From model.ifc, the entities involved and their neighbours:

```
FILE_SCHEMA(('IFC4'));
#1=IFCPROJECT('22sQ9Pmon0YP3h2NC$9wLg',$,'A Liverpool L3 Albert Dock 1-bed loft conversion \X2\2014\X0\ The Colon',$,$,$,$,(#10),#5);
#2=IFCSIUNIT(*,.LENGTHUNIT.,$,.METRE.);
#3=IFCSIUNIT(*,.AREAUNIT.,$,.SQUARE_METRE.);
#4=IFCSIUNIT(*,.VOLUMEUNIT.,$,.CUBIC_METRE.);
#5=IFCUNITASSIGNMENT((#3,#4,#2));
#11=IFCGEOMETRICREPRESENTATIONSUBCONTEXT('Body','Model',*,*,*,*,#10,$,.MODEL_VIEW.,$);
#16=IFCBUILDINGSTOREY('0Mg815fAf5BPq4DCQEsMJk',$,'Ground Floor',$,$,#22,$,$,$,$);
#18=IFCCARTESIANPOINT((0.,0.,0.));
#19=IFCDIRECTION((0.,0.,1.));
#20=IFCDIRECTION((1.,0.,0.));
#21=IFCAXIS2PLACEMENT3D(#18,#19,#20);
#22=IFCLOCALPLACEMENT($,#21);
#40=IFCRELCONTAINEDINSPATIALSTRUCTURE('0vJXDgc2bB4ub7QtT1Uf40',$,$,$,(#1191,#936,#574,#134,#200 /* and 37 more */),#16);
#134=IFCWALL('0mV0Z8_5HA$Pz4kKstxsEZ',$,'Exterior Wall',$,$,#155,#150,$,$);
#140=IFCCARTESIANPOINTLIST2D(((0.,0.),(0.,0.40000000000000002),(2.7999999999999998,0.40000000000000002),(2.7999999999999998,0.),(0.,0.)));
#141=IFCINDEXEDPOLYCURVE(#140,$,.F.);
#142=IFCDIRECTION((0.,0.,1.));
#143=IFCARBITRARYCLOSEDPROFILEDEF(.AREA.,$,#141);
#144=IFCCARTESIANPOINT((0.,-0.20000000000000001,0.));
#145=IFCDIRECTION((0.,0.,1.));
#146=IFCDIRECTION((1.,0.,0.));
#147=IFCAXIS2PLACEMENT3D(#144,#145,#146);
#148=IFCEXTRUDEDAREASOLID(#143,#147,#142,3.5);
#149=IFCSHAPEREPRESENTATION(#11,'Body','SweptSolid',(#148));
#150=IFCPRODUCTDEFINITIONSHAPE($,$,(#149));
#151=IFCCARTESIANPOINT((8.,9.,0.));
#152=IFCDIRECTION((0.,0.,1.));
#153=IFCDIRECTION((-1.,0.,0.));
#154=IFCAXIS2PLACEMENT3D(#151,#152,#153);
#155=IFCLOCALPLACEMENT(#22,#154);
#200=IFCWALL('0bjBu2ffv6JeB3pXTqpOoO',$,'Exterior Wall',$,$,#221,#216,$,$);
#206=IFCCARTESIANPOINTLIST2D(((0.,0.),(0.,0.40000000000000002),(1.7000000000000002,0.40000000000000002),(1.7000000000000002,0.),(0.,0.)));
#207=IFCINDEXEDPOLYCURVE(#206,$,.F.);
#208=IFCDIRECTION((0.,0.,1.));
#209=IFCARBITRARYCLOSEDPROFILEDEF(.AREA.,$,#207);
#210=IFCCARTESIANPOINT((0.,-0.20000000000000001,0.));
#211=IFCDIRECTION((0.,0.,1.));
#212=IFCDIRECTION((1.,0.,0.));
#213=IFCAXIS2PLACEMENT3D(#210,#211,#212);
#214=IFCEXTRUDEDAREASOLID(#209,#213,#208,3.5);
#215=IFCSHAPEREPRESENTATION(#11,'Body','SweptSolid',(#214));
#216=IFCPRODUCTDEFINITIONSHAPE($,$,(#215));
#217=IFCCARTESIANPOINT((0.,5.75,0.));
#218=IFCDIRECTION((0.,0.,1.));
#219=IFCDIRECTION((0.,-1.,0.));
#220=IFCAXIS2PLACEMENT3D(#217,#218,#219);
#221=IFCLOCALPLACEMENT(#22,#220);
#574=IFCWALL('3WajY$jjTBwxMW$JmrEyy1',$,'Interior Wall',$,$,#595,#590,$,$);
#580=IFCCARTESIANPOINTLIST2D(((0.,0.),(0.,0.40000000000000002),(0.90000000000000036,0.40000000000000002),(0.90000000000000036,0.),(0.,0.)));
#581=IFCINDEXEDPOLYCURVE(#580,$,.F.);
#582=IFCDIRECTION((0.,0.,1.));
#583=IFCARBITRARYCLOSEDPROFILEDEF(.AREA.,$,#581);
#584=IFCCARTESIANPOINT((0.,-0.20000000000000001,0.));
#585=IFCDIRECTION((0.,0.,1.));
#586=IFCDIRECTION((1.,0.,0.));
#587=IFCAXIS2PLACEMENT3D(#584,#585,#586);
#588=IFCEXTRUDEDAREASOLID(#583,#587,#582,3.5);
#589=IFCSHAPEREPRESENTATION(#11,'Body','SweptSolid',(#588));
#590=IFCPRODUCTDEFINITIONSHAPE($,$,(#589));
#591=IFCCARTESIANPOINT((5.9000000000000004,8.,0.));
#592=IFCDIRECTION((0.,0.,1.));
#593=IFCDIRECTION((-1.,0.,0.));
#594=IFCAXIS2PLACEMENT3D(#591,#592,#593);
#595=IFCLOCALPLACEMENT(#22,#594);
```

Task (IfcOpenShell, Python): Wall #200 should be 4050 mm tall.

```python
import ifcopenshell
import ifcopenshell.geom
import ifcopenshell.util.representation
import ifcopenshell.util.shape
import ifcopenshell.util.unit

model = ifcopenshell.open("model.ifc")
unit_scale = ifcopenshell.util.unit.calculate_unit_scale(model)
settings = ifcopenshell.geom.settings()


def volume(element):
    """Net volume in cubic metres, openings subtracted."""
    shape = ifcopenshell.geom.create_shape(settings, element)
    return ifcopenshell.util.shape.get_volume(shape.geometry)


wall = model.by_guid("0bjBu2ffv6JeB3pXTqpOoO")
before = volume(wall)

body = ifcopenshell.util.representation.get_representation(wall, "Model", "Body")
solid = body.Items[0]
old_height = solid.Depth
solid.Depth = 4.05 / unit_scale
after = volume(wall)

print(f"height {old_height:g} -> {solid.Depth:g}, volume {before:.3f} -> {after:.3f} m3")

model.write("model_edited.ifc")
```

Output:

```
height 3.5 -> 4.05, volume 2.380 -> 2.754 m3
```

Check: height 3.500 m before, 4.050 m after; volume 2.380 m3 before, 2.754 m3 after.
